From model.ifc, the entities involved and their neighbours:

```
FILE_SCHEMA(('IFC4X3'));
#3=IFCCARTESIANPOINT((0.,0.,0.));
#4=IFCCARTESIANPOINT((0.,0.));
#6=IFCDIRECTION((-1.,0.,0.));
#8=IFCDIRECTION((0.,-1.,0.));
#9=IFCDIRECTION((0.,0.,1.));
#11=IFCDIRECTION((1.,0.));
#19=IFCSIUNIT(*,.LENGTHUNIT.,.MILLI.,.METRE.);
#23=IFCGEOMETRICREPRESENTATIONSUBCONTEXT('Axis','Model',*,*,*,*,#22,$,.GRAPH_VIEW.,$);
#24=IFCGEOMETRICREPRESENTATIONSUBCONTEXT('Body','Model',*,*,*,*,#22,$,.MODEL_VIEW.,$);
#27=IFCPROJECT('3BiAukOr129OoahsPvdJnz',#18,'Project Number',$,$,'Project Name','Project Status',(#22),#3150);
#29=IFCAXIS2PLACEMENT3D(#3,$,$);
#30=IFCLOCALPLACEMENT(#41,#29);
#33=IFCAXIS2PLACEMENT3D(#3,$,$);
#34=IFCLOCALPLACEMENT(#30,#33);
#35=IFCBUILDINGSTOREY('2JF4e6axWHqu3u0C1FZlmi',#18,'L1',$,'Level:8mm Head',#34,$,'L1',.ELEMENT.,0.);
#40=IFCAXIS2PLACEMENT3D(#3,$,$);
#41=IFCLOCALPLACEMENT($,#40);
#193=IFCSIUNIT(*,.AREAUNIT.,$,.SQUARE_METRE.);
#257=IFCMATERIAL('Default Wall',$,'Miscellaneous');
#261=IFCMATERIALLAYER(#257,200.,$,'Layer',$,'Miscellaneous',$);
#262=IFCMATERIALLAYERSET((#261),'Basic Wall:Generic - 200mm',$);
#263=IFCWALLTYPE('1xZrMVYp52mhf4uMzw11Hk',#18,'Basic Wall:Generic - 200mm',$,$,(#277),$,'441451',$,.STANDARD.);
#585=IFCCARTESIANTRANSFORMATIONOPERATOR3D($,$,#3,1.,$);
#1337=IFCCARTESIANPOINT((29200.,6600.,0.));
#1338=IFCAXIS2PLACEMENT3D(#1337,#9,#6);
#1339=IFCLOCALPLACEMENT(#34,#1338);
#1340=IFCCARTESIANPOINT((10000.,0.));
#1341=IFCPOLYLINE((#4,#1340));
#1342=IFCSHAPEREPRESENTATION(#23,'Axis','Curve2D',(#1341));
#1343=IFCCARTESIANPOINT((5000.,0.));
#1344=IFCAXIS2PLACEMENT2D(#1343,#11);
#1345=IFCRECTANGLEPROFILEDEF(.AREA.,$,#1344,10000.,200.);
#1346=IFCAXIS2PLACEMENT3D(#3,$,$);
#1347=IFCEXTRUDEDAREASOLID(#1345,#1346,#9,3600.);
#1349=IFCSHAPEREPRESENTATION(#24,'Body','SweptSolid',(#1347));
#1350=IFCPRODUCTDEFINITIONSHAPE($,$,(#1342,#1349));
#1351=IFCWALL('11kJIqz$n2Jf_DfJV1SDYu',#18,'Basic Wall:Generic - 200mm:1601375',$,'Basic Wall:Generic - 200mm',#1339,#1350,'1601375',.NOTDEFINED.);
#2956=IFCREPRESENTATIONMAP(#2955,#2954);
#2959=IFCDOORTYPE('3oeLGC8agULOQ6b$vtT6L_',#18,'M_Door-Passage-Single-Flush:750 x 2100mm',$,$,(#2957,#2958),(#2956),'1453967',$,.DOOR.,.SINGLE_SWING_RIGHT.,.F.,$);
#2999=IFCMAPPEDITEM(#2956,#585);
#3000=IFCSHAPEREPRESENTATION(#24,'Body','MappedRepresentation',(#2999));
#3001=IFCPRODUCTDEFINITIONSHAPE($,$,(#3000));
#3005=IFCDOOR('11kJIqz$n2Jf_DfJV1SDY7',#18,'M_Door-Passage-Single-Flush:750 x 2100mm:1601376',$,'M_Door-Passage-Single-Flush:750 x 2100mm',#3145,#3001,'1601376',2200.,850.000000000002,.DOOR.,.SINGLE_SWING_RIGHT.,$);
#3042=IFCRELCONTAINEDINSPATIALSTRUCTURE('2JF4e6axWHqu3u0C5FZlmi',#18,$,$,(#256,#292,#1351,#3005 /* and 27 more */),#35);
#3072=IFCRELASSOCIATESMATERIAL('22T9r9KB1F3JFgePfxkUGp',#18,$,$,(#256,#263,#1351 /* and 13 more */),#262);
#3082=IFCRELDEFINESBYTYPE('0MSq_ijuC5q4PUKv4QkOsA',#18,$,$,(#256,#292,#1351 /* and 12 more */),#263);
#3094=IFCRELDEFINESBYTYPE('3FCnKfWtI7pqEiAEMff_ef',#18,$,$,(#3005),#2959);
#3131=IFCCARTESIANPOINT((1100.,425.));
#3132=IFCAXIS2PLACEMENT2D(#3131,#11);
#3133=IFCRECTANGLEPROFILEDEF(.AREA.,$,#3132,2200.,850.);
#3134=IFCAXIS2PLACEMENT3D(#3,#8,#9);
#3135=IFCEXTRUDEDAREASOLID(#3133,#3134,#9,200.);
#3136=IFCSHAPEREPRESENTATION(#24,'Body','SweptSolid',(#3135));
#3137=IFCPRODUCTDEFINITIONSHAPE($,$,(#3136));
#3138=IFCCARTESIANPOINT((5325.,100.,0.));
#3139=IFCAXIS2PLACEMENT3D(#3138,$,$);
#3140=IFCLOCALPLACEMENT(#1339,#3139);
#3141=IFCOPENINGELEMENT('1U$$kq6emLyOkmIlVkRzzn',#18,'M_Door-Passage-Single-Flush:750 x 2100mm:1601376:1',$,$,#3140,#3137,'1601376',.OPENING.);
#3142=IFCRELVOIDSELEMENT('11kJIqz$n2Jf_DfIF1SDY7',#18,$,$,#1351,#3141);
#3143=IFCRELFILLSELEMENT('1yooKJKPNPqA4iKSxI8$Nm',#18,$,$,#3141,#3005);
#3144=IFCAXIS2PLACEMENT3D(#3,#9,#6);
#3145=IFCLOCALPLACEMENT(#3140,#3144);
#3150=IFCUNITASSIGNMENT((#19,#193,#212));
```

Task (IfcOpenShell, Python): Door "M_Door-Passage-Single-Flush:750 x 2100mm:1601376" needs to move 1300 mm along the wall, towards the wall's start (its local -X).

```python
import ifcopenshell
import ifcopenshell.api.geometry
import ifcopenshell.util.placement
import ifcopenshell.util.unit

model = ifcopenshell.open("model.ifc")
unit_scale = ifcopenshell.util.unit.calculate_unit_scale(model)

door = model.by_guid("11kJIqz$n2Jf_DfJV1SDY7")
opening = door.FillsVoids[0].RelatingOpeningElement
wall = opening.VoidsElements[0].RelatingBuildingElement

wall_matrix = ifcopenshell.util.placement.get_local_placement(wall.ObjectPlacement)
shift = wall_matrix[:3, 0] * -1.3 / unit_scale
before = ifcopenshell.util.placement.get_local_placement(door.ObjectPlacement)[:3, 3].copy()

# The door is placed relative to its opening, so it follows when the opening moves.
matrix = ifcopenshell.util.placement.get_local_placement(opening.ObjectPlacement)
matrix[:3, 3] += shift
ifcopenshell.api.geometry.edit_object_placement(
    model, product=opening, matrix=matrix, is_si=False, should_transform_children=True
)

after = ifcopenshell.util.placement.get_local_placement(door.ObjectPlacement)[:3, 3]
print("door moved by", (after - before).round(3) + 0.0)

model.write("model-out.ifc")
```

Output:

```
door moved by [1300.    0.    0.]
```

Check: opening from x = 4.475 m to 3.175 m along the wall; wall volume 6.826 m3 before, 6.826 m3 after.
